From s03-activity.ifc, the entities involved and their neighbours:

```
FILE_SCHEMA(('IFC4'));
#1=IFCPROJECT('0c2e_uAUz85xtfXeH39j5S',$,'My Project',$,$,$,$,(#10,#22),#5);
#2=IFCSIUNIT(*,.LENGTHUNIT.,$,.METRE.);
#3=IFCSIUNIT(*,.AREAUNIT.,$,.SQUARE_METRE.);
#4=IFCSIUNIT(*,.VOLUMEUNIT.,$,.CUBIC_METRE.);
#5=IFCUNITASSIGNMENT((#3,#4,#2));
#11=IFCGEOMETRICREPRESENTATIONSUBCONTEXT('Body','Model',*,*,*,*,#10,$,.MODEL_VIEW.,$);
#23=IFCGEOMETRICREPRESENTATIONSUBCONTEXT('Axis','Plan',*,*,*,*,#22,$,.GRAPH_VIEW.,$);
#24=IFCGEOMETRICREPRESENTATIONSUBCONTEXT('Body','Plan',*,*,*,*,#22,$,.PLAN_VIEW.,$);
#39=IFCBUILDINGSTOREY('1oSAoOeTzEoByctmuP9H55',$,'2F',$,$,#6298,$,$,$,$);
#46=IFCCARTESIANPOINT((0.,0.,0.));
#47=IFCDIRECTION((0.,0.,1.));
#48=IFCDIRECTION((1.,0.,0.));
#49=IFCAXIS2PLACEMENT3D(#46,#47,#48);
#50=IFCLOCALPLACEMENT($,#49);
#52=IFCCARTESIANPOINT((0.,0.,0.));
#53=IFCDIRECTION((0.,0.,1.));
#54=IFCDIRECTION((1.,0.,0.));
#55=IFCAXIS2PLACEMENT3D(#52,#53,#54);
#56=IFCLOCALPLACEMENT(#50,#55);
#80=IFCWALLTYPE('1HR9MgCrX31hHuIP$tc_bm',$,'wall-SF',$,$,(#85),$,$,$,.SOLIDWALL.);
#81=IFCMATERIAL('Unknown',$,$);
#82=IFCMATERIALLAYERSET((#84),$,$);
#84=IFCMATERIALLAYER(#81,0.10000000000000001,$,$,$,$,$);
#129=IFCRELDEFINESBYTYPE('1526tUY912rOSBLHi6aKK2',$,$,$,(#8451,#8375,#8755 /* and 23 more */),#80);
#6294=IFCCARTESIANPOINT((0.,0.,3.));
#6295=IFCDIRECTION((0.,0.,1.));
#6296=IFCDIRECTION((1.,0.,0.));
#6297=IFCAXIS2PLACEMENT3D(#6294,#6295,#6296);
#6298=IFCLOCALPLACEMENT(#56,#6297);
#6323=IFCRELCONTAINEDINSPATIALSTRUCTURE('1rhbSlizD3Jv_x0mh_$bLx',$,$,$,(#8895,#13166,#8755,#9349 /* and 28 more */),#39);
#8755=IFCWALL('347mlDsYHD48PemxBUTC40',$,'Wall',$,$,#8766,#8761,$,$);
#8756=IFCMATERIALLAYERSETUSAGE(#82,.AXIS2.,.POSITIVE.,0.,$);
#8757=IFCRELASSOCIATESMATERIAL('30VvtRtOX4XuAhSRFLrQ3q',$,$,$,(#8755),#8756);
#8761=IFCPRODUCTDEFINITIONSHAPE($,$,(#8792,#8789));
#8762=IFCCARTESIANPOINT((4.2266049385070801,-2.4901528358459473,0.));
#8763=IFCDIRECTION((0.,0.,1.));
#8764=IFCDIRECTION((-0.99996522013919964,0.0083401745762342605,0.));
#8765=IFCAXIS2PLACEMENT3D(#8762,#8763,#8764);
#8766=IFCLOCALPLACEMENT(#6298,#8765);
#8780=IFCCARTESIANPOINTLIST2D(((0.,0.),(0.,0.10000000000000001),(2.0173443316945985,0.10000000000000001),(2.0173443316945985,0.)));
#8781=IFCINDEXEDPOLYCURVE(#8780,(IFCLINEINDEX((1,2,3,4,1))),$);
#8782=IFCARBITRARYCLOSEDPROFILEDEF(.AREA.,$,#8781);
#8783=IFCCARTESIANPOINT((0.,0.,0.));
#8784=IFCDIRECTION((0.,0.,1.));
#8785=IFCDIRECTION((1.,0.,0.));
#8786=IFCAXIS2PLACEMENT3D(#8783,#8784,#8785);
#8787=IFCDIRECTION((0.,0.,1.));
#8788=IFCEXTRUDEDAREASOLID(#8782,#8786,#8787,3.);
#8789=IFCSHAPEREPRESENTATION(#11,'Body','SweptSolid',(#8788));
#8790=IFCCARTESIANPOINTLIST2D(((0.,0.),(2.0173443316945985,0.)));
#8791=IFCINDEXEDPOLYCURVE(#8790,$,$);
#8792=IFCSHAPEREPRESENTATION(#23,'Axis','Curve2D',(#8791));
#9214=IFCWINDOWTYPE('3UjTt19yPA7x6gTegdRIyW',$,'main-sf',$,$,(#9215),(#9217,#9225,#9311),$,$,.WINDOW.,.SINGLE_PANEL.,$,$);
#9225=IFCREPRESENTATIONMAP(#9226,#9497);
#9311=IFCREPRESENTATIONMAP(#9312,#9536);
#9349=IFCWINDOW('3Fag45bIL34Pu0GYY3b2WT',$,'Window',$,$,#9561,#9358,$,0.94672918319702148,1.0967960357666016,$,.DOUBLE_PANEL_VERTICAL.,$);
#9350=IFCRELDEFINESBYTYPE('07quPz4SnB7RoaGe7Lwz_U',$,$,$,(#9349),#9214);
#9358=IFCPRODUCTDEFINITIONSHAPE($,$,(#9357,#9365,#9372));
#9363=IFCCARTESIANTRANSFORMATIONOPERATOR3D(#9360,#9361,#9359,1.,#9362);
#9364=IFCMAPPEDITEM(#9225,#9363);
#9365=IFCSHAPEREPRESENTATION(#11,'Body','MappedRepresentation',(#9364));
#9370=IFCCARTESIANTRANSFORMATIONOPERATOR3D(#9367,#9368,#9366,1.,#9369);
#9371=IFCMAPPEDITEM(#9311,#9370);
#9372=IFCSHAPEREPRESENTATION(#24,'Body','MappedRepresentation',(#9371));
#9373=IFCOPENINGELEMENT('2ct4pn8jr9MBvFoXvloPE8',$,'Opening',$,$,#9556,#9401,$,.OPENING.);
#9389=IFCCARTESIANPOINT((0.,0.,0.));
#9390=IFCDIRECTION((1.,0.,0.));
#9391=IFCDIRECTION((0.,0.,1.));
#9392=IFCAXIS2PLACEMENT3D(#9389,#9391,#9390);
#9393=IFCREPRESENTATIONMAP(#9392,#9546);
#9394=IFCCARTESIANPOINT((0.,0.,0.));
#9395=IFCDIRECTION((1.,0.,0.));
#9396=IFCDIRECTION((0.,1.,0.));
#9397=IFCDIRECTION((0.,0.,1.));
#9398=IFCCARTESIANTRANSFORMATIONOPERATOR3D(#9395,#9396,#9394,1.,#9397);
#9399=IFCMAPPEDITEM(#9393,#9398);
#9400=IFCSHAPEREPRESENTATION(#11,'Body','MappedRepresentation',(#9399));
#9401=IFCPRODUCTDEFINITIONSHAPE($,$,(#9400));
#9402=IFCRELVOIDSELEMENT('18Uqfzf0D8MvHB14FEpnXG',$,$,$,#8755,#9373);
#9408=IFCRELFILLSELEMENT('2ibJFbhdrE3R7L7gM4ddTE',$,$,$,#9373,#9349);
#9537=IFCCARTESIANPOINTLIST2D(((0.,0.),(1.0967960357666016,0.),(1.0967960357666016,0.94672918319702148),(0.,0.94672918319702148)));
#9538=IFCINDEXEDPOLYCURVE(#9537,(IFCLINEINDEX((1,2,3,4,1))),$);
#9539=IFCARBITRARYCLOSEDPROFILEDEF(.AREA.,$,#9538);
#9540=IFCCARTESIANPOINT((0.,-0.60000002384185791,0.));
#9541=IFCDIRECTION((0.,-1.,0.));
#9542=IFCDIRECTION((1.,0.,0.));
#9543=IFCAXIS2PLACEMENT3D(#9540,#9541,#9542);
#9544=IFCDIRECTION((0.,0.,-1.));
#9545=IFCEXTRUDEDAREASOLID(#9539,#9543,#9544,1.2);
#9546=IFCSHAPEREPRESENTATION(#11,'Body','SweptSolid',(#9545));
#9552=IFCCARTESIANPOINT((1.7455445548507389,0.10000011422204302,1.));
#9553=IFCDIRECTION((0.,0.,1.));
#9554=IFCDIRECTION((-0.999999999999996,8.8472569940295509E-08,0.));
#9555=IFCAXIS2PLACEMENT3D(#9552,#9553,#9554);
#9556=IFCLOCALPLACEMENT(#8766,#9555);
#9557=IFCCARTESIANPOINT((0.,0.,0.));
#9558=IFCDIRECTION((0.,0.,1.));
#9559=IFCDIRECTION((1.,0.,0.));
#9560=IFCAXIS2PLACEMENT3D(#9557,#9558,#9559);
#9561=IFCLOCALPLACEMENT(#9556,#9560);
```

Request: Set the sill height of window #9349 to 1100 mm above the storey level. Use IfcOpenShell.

```python
import numpy as np
import ifcopenshell
import ifcopenshell.api.geometry
import ifcopenshell.geom
import ifcopenshell.util.element
import ifcopenshell.util.placement
import ifcopenshell.util.shape
import ifcopenshell.util.unit

model = ifcopenshell.open("s03-activity.ifc")
unit_scale = ifcopenshell.util.unit.calculate_unit_scale(model)

window = model.by_id(9349)
opening = window.FillsVoids[0].RelatingOpeningElement
storey = ifcopenshell.util.element.get_container(window, ifc_class="IfcBuildingStorey")
level = ifcopenshell.util.placement.get_local_placement(storey.ObjectPlacement)[2, 3]

# The opening's origin need not be at the sill, so measure its lowest point.
shape = ifcopenshell.geom.create_shape(ifcopenshell.geom.settings(), opening)
bottom = ifcopenshell.util.shape.get_shape_bottom_elevation(shape, shape.geometry) / unit_scale
dz = level + 1.1 - bottom

shift = np.array([0.0, 0.0, dz])
# The window is placed relative to its opening, so it follows when the opening moves.
matrix = ifcopenshell.util.placement.get_local_placement(opening.ObjectPlacement)
matrix[:3, 3] += shift
ifcopenshell.api.geometry.edit_object_placement(
    model, product=opening, matrix=matrix, is_si=False, should_transform_children=True
)

print(f"moved by {dz * unit_scale:+.3f} m")

model.write("s03-activity-out.ifc")
```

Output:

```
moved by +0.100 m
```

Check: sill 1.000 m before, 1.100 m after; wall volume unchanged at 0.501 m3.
